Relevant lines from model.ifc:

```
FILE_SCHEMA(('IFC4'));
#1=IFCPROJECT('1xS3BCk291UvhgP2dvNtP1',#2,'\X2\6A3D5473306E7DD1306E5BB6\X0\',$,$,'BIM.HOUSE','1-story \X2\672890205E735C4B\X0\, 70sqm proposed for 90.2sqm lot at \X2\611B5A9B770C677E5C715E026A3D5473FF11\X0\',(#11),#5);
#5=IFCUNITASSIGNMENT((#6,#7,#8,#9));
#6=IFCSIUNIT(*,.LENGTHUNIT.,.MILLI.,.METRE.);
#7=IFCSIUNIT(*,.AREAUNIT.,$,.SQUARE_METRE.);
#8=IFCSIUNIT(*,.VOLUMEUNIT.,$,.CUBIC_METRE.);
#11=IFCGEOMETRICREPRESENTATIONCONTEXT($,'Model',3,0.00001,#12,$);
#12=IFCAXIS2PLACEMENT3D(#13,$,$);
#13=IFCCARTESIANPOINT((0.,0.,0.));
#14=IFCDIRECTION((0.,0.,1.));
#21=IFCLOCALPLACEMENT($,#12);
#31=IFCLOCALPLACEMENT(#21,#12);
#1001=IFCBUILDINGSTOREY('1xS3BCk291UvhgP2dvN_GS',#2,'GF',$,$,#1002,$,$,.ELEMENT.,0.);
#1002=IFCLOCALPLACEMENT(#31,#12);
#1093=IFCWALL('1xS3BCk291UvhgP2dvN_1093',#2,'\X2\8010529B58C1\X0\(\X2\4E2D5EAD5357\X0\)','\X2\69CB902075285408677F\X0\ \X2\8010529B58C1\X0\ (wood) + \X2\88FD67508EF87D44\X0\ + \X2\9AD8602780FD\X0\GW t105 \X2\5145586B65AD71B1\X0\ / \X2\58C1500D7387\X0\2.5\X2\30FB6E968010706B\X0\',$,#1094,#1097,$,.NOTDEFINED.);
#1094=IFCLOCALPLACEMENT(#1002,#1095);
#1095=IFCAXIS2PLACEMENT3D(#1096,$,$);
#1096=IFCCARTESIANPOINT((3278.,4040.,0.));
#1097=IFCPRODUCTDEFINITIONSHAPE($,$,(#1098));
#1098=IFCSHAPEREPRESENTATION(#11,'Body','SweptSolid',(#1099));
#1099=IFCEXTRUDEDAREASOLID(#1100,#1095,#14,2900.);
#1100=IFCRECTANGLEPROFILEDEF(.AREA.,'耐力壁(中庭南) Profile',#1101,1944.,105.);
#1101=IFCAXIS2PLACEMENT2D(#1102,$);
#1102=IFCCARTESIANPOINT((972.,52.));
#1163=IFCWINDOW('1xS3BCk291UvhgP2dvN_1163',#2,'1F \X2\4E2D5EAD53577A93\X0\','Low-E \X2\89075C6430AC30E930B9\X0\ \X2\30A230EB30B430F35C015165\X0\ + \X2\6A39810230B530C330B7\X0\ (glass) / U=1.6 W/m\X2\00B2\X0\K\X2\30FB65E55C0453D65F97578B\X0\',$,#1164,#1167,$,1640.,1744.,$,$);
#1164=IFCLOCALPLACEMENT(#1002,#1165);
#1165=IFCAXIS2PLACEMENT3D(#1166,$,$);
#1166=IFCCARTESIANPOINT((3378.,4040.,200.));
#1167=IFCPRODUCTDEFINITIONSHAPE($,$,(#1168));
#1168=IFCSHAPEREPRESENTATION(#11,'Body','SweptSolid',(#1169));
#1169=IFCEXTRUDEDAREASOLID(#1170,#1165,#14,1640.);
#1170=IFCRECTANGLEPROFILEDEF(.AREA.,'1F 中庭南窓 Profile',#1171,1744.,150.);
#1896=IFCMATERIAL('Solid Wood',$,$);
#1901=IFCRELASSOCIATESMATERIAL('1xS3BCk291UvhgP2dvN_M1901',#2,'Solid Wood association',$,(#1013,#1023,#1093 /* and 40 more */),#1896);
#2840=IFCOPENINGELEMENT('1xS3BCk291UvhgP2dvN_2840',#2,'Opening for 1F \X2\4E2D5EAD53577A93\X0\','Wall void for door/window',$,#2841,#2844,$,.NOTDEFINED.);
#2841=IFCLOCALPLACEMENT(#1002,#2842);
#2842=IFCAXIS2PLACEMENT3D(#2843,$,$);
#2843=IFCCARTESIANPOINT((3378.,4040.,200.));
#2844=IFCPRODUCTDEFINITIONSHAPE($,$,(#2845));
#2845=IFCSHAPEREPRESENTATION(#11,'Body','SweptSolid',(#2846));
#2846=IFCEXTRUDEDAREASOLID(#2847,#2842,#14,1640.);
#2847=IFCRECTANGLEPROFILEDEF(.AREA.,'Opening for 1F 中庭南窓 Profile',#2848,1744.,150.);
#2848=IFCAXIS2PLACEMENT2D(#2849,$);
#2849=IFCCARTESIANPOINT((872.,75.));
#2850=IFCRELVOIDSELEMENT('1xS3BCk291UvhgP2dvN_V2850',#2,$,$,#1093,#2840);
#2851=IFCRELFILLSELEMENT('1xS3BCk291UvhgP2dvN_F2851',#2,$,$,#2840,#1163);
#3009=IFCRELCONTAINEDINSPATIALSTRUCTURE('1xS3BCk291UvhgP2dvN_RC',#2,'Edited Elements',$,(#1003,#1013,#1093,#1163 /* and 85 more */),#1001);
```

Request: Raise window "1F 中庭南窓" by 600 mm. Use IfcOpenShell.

```python
import numpy as np
import ifcopenshell
import ifcopenshell.api.geometry
import ifcopenshell.util.placement
import ifcopenshell.util.unit

model = ifcopenshell.open("model.ifc")
unit_scale = ifcopenshell.util.unit.calculate_unit_scale(model)

window = model.by_guid("1xS3BCk291UvhgP2dvN_1163")
opening = window.FillsVoids[0].RelatingOpeningElement
dz = 0.6 / unit_scale

shift = np.array([0.0, 0.0, dz])
# The window is not placed relative to its opening, so move both.
for product in (opening, window):
    matrix = ifcopenshell.util.placement.get_local_placement(product.ObjectPlacement)
    matrix[:3, 3] += shift
    ifcopenshell.api.geometry.edit_object_placement(model, product=product, matrix=matrix, is_si=False)

print(f"moved by {dz * unit_scale:+.3f} m")

model.write("model-out.ifc")
```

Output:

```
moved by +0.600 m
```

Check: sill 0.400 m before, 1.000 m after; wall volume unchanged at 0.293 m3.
